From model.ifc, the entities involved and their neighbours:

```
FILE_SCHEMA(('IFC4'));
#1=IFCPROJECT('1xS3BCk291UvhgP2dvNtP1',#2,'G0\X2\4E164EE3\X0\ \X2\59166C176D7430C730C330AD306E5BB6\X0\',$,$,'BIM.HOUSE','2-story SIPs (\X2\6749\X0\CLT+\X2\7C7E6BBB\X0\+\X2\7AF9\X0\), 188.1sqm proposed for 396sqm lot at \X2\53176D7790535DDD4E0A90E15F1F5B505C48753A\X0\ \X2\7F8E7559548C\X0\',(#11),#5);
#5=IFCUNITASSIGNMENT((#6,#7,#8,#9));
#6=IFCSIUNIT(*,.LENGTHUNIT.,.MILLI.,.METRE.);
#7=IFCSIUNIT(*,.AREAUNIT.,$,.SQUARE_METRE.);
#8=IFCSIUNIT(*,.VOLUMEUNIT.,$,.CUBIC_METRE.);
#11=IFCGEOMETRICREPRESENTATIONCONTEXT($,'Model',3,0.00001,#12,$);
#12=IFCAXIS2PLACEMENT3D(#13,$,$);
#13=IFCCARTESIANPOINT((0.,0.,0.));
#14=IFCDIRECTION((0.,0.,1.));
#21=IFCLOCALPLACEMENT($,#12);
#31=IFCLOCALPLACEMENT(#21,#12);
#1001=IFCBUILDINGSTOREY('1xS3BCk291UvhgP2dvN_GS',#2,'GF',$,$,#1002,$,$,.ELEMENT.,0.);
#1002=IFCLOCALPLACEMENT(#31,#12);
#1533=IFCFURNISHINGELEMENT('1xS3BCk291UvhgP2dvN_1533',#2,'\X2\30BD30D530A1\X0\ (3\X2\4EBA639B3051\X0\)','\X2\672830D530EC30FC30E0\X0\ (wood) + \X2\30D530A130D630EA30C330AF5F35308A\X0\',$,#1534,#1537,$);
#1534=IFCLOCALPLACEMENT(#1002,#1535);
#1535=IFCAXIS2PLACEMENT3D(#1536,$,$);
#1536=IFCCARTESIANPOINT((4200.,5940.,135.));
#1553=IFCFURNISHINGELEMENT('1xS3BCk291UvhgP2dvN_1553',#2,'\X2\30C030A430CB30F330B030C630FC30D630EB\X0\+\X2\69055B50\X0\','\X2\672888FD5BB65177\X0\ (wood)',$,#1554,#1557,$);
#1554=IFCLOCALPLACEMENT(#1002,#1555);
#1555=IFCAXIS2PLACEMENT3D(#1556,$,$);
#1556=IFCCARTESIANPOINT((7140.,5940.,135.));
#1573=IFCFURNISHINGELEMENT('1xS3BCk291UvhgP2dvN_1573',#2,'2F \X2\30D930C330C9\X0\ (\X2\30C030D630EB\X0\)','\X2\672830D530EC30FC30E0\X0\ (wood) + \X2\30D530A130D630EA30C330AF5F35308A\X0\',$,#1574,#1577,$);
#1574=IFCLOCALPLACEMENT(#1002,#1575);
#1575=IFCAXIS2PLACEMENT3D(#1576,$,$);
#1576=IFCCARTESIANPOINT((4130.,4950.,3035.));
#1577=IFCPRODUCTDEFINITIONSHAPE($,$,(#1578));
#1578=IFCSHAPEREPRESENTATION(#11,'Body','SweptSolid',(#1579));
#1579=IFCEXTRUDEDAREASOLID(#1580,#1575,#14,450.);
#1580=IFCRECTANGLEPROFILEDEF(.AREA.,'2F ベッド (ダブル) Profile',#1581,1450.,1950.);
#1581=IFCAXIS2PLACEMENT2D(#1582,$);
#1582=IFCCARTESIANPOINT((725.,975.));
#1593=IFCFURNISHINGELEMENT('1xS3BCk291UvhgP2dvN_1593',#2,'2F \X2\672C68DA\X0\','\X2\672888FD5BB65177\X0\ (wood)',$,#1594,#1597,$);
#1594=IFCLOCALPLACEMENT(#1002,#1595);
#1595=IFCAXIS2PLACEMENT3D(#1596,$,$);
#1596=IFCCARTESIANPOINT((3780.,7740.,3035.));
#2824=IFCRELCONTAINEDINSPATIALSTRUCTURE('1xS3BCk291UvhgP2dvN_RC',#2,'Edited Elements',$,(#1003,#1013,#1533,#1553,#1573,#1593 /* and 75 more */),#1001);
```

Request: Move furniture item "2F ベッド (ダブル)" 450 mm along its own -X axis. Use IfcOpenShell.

```python
import ifcopenshell
import ifcopenshell.api.geometry
import ifcopenshell.util.placement
import ifcopenshell.util.unit

model = ifcopenshell.open("model.ifc")
unit_scale = ifcopenshell.util.unit.calculate_unit_scale(model)

item = model.by_guid("1xS3BCk291UvhgP2dvN_1573")
matrix = ifcopenshell.util.placement.get_local_placement(item.ObjectPlacement)
matrix[:3, 3] -= matrix[:3, 0] * 0.45 / unit_scale
ifcopenshell.api.geometry.edit_object_placement(model, product=item, matrix=matrix, is_si=False)

print(ifcopenshell.util.placement.get_local_placement(item.ObjectPlacement).round(3) + 0.0)

model.write("model-out.ifc")
```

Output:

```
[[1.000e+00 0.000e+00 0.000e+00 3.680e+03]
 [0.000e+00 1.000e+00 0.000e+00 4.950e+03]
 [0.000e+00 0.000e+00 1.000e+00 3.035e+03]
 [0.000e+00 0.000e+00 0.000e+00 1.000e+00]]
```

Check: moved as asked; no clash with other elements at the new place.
